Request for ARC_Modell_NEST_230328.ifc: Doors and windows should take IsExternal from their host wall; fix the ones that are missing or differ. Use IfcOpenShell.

First a look at what the model holds.

```python
import ifcopenshell
import ifcopenshell.util.element

model = ifcopenshell.open("ARC_Modell_NEST_230328.ifc")
print(model.schema)
seen = {}
for e in model.by_type("IfcDoor") + model.by_type("IfcWindow"):
    if not e.FillsVoids:
        continue
    host = e.FillsVoids[0].RelatingOpeningElement.VoidsElements[0].RelatingBuildingElement
    own = ifcopenshell.util.element.get_pset(e, f"Pset_{e.is_a()[3:].removesuffix('StandardCase')}Common", "IsExternal")
    wall = ifcopenshell.util.element.get_pset(host, "Pset_WallCommon", "IsExternal")
    seen[e.is_a(), own, wall] = seen.get((e.is_a(), own, wall), 0) + 1
for (cls, own, wall), count in sorted(seen.items(), key=str):
    print(count, cls, "IsExternal:", own, "| host wall:", wall)
```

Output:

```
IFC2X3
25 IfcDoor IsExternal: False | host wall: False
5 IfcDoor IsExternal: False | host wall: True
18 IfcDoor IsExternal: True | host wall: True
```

```python
import ifcopenshell
import ifcopenshell.api.pset
import ifcopenshell.util.element

model = ifcopenshell.open("ARC_Modell_NEST_230328.ifc")

count = 0
for ifc_class, pset_name in (("IfcDoor", "Pset_DoorCommon"), ("IfcWindow", "Pset_WindowCommon")):
    for e in model.by_type(ifc_class):
        if not e.FillsVoids:
            continue
        host = e.FillsVoids[0].RelatingOpeningElement.VoidsElements[0].RelatingBuildingElement
        external = ifcopenshell.util.element.get_pset(host, "Pset_WallCommon", "IsExternal")
        if external is None or ifcopenshell.util.element.get_pset(e, pset_name, "IsExternal") == external:
            continue
        pset = ifcopenshell.api.pset.add_pset(model, product=e, name=pset_name)
        ifcopenshell.api.pset.edit_pset(model, pset=pset, properties={"IsExternal": external})
        count += 1

print(count, "updated")

model.write("ARC_Modell_NEST_230328_v2.ifc")
```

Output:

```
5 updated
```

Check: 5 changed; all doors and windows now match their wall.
